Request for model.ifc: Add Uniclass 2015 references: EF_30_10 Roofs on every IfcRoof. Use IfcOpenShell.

First a look at what the model holds.

```python
import ifcopenshell

model = ifcopenshell.open("model.ifc")
print(model.schema)
print("classifications:", [c.Name for c in model.by_type("IfcClassification")])
for ifc_class in ("IfcDoor", "IfcRoof", "IfcStair", "IfcWall", "IfcWindow"):
    print(ifc_class, len(model.by_type(ifc_class)))
```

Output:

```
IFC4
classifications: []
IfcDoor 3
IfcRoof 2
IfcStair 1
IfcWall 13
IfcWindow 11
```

```python
import ifcopenshell
import ifcopenshell.api.classification

model = ifcopenshell.open("model.ifc")

system = ifcopenshell.api.classification.add_classification(model, classification="Uniclass 2015")

codes = {
    "IfcRoof": ("EF_30_10", "Roofs"),
}
for ifc_class, (code, name) in codes.items():
    products = model.by_type(ifc_class)
    ifcopenshell.api.classification.add_reference(
        model, products=products, classification=system, identification=code, name=name
    )
    print(code, len(products))

model.write("model_v2.ifc")
```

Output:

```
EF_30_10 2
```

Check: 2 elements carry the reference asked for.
